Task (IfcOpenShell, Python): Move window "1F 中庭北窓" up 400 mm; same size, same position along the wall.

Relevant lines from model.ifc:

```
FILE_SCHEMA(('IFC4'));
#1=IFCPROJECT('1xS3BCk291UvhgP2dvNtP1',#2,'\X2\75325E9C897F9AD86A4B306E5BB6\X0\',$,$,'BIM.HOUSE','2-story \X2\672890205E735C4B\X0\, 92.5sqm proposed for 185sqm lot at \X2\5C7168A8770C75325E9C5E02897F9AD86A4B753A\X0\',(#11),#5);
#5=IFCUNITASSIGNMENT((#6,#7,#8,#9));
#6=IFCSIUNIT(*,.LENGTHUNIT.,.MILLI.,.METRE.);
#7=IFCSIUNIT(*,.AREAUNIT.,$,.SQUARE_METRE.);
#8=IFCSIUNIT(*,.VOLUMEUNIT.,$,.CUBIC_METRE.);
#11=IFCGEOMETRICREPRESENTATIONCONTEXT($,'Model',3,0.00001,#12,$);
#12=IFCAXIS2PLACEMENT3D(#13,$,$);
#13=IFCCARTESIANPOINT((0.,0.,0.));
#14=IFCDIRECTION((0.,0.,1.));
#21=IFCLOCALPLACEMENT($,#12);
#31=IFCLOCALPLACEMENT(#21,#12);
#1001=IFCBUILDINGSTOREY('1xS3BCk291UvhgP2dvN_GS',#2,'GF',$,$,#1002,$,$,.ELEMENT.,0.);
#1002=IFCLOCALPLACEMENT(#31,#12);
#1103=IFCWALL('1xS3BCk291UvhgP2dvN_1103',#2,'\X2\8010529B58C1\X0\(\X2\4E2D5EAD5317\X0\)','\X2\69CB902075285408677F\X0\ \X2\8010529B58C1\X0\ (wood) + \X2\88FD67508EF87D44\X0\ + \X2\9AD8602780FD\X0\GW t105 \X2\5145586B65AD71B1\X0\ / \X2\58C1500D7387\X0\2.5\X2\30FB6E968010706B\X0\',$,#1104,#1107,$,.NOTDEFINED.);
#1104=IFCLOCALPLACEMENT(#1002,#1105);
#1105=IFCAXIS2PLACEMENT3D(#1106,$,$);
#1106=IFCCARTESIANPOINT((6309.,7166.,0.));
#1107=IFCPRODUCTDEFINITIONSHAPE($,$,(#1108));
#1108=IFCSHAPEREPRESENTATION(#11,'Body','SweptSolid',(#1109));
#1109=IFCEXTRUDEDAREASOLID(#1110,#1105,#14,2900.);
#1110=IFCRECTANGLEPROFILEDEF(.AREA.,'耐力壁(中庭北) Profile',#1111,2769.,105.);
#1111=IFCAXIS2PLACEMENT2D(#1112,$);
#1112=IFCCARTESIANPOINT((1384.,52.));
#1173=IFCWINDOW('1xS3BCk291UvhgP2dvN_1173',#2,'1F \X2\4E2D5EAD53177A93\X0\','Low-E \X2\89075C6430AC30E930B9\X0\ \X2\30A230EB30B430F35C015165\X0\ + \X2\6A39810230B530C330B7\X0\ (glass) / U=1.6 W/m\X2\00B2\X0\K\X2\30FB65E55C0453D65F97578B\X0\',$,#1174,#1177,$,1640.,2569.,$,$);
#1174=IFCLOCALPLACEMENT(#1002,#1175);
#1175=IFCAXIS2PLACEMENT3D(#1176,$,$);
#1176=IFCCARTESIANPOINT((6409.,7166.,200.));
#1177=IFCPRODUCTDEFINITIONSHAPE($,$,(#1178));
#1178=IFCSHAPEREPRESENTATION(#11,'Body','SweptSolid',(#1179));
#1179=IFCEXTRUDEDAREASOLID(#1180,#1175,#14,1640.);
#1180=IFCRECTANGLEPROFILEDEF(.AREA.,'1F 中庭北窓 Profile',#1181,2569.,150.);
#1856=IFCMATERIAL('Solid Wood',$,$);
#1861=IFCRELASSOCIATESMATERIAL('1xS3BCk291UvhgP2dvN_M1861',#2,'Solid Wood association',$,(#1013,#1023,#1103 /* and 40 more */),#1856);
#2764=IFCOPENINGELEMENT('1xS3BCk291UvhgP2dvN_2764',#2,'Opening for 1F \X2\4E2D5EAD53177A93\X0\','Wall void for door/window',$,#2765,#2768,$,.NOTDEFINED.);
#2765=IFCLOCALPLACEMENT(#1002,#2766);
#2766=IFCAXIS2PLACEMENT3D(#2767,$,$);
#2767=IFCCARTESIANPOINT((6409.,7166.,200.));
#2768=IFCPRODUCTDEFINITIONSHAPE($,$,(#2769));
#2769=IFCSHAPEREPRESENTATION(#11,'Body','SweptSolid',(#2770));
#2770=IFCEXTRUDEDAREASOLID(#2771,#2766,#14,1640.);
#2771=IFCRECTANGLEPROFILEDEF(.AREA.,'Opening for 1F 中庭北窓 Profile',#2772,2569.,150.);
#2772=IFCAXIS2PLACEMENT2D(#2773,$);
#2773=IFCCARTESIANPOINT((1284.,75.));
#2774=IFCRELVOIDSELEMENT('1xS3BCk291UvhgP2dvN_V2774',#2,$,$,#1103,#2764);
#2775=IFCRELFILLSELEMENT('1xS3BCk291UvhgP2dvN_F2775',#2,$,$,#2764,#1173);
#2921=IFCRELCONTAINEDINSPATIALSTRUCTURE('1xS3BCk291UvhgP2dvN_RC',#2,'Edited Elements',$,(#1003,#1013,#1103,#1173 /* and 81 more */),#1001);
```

```python
import numpy as np
import ifcopenshell
import ifcopenshell.api.geometry
import ifcopenshell.util.placement
import ifcopenshell.util.unit

model = ifcopenshell.open("model.ifc")
unit_scale = ifcopenshell.util.unit.calculate_unit_scale(model)

window = model.by_guid("1xS3BCk291UvhgP2dvN_1173")
opening = window.FillsVoids[0].RelatingOpeningElement
dz = 0.4 / unit_scale

shift = np.array([0.0, 0.0, dz])
# The window is not placed relative to its opening, so move both.
for product in (opening, window):
    matrix = ifcopenshell.util.placement.get_local_placement(product.ObjectPlacement)
    matrix[:3, 3] += shift
    ifcopenshell.api.geometry.edit_object_placement(model, product=product, matrix=matrix, is_si=False)

print(f"moved by {dz * unit_scale:+.3f} m")

model.write("model_edited.ifc")
```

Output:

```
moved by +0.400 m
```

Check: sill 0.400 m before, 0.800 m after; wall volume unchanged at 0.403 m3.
